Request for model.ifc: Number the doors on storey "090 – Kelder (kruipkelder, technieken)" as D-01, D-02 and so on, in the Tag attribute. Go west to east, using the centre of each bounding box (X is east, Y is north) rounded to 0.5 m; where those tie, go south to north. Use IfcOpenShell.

First a look at what the model holds.

```python
import ifcopenshell
import ifcopenshell.util.element
import ifcopenshell.util.placement

model = ifcopenshell.open("model.ifc")
print(model.schema)
storey = next(s for s in model.by_type("IfcBuildingStorey") if s.Name == "090 – Kelder (kruipkelder, technieken)")
doors = [e for e in ifcopenshell.util.element.get_decomposition(storey) if e.is_a("IfcDoor")]
for e in sorted(doors, key=lambda e: e.id()):
    origin = ifcopenshell.util.placement.get_local_placement(e.ObjectPlacement)[:3, 3]
    print(e.id(), e.Tag, e.Name, origin.round(2) + 0.0, sep=" | ")
```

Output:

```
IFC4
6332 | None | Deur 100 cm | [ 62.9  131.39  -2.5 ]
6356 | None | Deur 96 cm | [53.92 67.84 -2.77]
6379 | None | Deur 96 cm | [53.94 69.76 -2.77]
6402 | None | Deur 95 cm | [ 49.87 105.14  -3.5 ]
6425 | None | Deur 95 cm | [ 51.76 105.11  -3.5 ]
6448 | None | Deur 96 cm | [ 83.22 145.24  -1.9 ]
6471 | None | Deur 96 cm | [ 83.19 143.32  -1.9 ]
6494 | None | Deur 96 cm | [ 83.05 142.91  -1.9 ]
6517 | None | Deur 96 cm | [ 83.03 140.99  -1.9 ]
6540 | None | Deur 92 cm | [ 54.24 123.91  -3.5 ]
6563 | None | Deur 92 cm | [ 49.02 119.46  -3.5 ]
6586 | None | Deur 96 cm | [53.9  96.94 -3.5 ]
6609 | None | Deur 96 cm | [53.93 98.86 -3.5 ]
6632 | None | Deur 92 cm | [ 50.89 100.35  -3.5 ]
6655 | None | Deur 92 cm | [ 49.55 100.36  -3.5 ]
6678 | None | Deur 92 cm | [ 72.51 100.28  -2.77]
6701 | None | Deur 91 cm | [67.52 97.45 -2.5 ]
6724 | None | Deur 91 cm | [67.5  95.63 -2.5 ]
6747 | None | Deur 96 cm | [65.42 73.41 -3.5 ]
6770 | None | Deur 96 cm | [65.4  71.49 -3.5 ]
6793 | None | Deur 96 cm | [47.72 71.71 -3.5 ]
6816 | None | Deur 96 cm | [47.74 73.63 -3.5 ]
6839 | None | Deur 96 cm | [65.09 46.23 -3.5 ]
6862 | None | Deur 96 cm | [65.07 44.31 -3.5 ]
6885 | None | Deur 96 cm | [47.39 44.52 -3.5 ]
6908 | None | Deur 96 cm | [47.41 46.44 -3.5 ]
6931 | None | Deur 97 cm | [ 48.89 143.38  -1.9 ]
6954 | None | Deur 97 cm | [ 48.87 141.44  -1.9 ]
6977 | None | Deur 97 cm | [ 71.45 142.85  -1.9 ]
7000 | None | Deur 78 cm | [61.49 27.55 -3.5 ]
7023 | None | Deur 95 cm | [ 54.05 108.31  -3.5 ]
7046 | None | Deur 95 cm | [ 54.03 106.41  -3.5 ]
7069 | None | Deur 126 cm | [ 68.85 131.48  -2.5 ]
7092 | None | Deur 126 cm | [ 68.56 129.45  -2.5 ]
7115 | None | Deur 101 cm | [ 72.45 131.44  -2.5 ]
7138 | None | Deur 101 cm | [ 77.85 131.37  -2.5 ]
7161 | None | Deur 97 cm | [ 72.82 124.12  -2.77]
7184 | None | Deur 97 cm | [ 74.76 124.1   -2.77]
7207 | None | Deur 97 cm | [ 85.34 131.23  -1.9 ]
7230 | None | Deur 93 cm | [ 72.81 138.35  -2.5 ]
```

```python
import ifcopenshell
import ifcopenshell.geom
import ifcopenshell.util.element
import ifcopenshell.util.shape

model = ifcopenshell.open("model.ifc")
settings = ifcopenshell.geom.settings()
settings.set("use-world-coords", True)


def centre(element):
    shape = ifcopenshell.geom.create_shape(settings, element)
    return ifcopenshell.util.shape.get_bbox_centroid(shape.geometry)


storey = next(s for s in model.by_type("IfcBuildingStorey") if s.Name == "090 – Kelder (kruipkelder, technieken)")
doors = [e for e in ifcopenshell.util.element.get_decomposition(storey) if e.is_a("IfcDoor")]

# Insertion points can sit at a corner or the storey origin, so sort by the geometry (in metres).
centres = {e: centre(e) for e in doors}
doors.sort(key=lambda e: (round(centres[e][0] / 0.5), centres[e][1]))

for i, e in enumerate(doors, start=1):
    number = f"D-{i:02d}"
    e.Tag = number
    print(e.id(), number)

model.write("model_edited.ifc")
```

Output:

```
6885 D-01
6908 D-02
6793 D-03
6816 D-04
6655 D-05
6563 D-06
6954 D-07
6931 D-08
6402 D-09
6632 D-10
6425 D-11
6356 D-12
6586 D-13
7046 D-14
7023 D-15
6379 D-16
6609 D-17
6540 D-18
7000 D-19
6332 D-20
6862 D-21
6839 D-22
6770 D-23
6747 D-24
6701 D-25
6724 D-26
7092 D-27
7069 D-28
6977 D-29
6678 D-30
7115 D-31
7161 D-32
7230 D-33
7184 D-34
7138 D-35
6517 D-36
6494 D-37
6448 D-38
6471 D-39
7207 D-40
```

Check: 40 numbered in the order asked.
